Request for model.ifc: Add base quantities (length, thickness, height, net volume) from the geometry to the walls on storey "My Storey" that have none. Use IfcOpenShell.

First a look at what the model holds.

```python
import ifcopenshell
import ifcopenshell.util.element
import ifcopenshell.util.unit

model = ifcopenshell.open("model.ifc")
print(model.schema)
for unit_type in ("LENGTHUNIT", "AREAUNIT", "VOLUMEUNIT"):
    print(unit_type, ifcopenshell.util.unit.calculate_unit_scale(model, unit_type))
storey = next(s for s in model.by_type("IfcBuildingStorey") if s.Name == "My Storey")
walls = [e for e in ifcopenshell.util.element.get_decomposition(storey) if e.is_a("IfcWall")]
for e in sorted(walls, key=lambda e: e.id()):
    print(e.id(), e.is_a(), e.Name, list(ifcopenshell.util.element.get_psets(e, qtos_only=True)), sep=" | ")
```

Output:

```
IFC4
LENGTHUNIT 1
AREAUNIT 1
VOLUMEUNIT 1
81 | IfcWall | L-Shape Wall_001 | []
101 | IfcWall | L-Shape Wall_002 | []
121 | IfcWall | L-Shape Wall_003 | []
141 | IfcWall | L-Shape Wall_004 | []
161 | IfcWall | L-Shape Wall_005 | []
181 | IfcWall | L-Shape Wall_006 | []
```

```python
import ifcopenshell
import ifcopenshell.api.pset
import ifcopenshell.geom
import ifcopenshell.util.element
import ifcopenshell.util.shape
import ifcopenshell.util.unit

model = ifcopenshell.open("model.ifc")
unit_scale = ifcopenshell.util.unit.calculate_unit_scale(model)
volume_scale = ifcopenshell.util.unit.calculate_unit_scale(model, "VOLUMEUNIT")
settings = ifcopenshell.geom.settings()

storey = next(s for s in model.by_type("IfcBuildingStorey") if s.Name == "My Storey")
walls = [e for e in ifcopenshell.util.element.get_decomposition(storey) if e.is_a("IfcWall")]

for e in sorted(walls, key=lambda e: e.id()):
    if ifcopenshell.util.element.get_psets(e, qtos_only=True, should_inherit=False):
        continue
    # Geometry comes back in metres, in the element's own axes.
    shape = ifcopenshell.geom.create_shape(settings, e)
    values = {
        "Length": ifcopenshell.util.shape.get_x(shape.geometry) / unit_scale,
        "Width": ifcopenshell.util.shape.get_y(shape.geometry) / unit_scale,
        "Height": ifcopenshell.util.shape.get_z(shape.geometry) / unit_scale,
        "NetVolume": ifcopenshell.util.shape.get_volume(shape.geometry) / volume_scale,
    }
    qto = ifcopenshell.api.pset.add_qto(model, product=e, name="Qto_WallBaseQuantities")
    ifcopenshell.api.pset.edit_qto(model, qto=qto, properties=values)
    print(e.id(), {k: round(v, 3) for k, v in values.items()})

model.write("model-out.ifc")
```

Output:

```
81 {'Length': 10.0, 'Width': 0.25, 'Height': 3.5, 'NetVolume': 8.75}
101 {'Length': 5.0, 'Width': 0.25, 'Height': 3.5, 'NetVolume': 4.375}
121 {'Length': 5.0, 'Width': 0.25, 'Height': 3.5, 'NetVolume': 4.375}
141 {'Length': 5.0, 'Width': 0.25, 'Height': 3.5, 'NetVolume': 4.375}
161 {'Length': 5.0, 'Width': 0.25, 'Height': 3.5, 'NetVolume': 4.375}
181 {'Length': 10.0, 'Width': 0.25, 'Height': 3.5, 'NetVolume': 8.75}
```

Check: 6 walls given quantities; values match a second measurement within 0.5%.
